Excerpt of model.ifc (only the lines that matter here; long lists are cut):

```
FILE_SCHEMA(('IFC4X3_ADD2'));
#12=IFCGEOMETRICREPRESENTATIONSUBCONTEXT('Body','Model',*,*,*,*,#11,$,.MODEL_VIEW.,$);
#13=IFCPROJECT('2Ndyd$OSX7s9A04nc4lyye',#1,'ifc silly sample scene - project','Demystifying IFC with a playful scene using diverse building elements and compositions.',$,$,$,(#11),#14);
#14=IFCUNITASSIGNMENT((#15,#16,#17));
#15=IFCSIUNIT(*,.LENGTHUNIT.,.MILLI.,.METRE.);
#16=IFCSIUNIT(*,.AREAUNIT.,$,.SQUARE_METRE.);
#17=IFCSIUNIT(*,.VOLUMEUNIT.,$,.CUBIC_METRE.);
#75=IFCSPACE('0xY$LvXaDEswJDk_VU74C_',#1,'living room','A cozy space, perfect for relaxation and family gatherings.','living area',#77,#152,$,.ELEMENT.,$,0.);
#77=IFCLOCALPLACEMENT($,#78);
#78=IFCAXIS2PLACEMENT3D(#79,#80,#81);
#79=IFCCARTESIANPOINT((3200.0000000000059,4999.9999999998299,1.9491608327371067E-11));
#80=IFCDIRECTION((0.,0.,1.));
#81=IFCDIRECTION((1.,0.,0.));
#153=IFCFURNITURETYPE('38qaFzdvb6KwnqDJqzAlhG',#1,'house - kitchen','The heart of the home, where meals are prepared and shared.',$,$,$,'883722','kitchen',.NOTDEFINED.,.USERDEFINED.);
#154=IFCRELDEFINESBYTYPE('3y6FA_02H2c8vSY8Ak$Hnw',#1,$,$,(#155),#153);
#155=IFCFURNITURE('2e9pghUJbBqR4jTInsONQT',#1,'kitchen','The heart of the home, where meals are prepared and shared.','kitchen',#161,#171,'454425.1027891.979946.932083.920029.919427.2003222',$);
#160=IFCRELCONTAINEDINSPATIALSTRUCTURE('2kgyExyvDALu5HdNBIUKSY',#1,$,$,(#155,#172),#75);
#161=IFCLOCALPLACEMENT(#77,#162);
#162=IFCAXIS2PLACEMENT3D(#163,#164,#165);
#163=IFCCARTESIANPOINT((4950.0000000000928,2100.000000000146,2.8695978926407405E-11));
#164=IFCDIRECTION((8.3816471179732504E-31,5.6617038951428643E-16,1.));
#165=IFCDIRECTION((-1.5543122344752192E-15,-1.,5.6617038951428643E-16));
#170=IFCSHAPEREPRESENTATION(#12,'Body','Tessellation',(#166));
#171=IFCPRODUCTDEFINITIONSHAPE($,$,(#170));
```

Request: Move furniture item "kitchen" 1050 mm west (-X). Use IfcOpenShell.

```python
import ifcopenshell
import ifcopenshell.api.geometry
import ifcopenshell.util.placement
import ifcopenshell.util.unit

model = ifcopenshell.open("model.ifc")
unit_scale = ifcopenshell.util.unit.calculate_unit_scale(model)

item = model.by_id(155)
matrix = ifcopenshell.util.placement.get_local_placement(item.ObjectPlacement)
matrix[0, 3] -= 1.05 / unit_scale
ifcopenshell.api.geometry.edit_object_placement(model, product=item, matrix=matrix, is_si=False)

print(ifcopenshell.util.placement.get_local_placement(item.ObjectPlacement).round(3) + 0.0)

model.write("model-out.ifc")
```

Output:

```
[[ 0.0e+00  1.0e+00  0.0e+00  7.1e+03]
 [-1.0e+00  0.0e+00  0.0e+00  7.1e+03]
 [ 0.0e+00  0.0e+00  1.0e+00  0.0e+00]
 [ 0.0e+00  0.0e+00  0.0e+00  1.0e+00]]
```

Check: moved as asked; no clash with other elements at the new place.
